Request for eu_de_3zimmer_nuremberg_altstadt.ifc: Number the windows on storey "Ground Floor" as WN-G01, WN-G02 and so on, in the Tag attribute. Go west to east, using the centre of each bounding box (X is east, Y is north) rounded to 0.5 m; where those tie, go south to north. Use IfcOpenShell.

First a look at what the model holds.

```python
import ifcopenshell
import ifcopenshell.util.element
import ifcopenshell.util.placement

model = ifcopenshell.open("eu_de_3zimmer_nuremberg_altstadt.ifc")
print(model.schema)
storey = next(s for s in model.by_type("IfcBuildingStorey") if s.Name == "Ground Floor")
windows = [e for e in ifcopenshell.util.element.get_decomposition(storey) if e.is_a("IfcWindow")]
for e in sorted(windows, key=lambda e: e.id()):
    origin = ifcopenshell.util.placement.get_local_placement(e.ObjectPlacement)[:3, 3]
    print(e.id(), e.Tag, e.Name, origin.round(2) + 0.0, sep=" | ")
```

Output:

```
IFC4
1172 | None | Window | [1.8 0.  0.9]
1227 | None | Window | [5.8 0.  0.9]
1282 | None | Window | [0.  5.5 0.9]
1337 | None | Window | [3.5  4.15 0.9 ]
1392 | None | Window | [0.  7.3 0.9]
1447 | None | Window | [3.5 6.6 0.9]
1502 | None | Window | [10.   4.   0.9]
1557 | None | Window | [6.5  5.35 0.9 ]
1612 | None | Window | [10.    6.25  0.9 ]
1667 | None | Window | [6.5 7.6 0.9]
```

```python
import ifcopenshell
import ifcopenshell.geom
import ifcopenshell.util.element
import ifcopenshell.util.shape

model = ifcopenshell.open("eu_de_3zimmer_nuremberg_altstadt.ifc")
settings = ifcopenshell.geom.settings()
settings.set("use-world-coords", True)


def centre(element):
    shape = ifcopenshell.geom.create_shape(settings, element)
    return ifcopenshell.util.shape.get_bbox_centroid(shape.geometry)


storey = next(s for s in model.by_type("IfcBuildingStorey") if s.Name == "Ground Floor")
windows = [e for e in ifcopenshell.util.element.get_decomposition(storey) if e.is_a("IfcWindow")]

# Insertion points can sit at a corner or the storey origin, so sort by the geometry (in metres).
centres = {e: centre(e) for e in windows}
windows.sort(key=lambda e: (round(centres[e][0] / 0.5), centres[e][1]))

for i, e in enumerate(windows, start=1):
    number = f"WN-G{i:02d}"
    e.Tag = number
    print(e.id(), number)

model.write("eu_de_3zimmer_nuremberg_altstadt-out.ifc")
```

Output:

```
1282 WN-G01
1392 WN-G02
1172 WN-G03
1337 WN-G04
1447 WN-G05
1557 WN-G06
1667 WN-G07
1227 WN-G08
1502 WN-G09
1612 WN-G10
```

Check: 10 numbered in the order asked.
